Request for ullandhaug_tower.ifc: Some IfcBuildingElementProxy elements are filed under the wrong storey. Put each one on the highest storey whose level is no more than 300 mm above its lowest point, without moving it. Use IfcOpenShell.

First a look at what the model holds.

```python
import ifcopenshell
import ifcopenshell.util.element
import ifcopenshell.util.placement

model = ifcopenshell.open("ullandhaug_tower.ifc")
print(model.schema)
for storey in model.by_type("IfcBuildingStorey"):
    level = ifcopenshell.util.placement.get_storey_elevation(storey)
    count = sum(e.is_a("IfcBuildingElementProxy") for e in ifcopenshell.util.element.get_contained(storey))
    print(storey.id(), storey.Name, round(level, 3), count, sep=" | ")
```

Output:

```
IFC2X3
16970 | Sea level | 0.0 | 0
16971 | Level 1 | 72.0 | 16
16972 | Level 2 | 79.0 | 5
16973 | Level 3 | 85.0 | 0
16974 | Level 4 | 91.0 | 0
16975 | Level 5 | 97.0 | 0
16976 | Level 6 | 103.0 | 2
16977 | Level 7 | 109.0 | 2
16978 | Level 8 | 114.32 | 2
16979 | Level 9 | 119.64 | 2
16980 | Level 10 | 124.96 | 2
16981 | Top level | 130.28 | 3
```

```python
import ifcopenshell
import ifcopenshell.api.spatial
import ifcopenshell.geom
import ifcopenshell.util.element
import ifcopenshell.util.placement
import ifcopenshell.util.shape
import ifcopenshell.util.unit

model = ifcopenshell.open("ullandhaug_tower.ifc")
unit_scale = ifcopenshell.util.unit.calculate_unit_scale(model)
settings = ifcopenshell.geom.settings()

levels = sorted(
    ((ifcopenshell.util.placement.get_storey_elevation(s) * unit_scale, s) for s in model.by_type("IfcBuildingStorey")),
    key=lambda pair: pair[0],
)

for e in model.by_type("IfcBuildingElementProxy"):
    current = e.ContainedInStructure[0].RelatingStructure if e.ContainedInStructure else None
    if current is None or not current.is_a("IfcBuildingStorey"):
        continue
    shape = ifcopenshell.geom.create_shape(settings, e)
    bottom = ifcopenshell.util.shape.get_shape_bottom_elevation(shape, shape.geometry)
    below = [s for level, s in levels if level <= bottom + 0.3]
    storey = below[-1] if below else levels[0][1]
    if storey != current:
        # assign_container keeps the world position.
        ifcopenshell.api.spatial.assign_container(model, products=[e], relating_structure=storey)
        print(e.id(), current.Name, "->", storey.Name)

model.write("ullandhaug_tower-out.ifc")
```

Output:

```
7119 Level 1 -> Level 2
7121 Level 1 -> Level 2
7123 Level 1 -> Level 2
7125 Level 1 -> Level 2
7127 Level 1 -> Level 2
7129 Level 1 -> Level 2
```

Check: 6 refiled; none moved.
